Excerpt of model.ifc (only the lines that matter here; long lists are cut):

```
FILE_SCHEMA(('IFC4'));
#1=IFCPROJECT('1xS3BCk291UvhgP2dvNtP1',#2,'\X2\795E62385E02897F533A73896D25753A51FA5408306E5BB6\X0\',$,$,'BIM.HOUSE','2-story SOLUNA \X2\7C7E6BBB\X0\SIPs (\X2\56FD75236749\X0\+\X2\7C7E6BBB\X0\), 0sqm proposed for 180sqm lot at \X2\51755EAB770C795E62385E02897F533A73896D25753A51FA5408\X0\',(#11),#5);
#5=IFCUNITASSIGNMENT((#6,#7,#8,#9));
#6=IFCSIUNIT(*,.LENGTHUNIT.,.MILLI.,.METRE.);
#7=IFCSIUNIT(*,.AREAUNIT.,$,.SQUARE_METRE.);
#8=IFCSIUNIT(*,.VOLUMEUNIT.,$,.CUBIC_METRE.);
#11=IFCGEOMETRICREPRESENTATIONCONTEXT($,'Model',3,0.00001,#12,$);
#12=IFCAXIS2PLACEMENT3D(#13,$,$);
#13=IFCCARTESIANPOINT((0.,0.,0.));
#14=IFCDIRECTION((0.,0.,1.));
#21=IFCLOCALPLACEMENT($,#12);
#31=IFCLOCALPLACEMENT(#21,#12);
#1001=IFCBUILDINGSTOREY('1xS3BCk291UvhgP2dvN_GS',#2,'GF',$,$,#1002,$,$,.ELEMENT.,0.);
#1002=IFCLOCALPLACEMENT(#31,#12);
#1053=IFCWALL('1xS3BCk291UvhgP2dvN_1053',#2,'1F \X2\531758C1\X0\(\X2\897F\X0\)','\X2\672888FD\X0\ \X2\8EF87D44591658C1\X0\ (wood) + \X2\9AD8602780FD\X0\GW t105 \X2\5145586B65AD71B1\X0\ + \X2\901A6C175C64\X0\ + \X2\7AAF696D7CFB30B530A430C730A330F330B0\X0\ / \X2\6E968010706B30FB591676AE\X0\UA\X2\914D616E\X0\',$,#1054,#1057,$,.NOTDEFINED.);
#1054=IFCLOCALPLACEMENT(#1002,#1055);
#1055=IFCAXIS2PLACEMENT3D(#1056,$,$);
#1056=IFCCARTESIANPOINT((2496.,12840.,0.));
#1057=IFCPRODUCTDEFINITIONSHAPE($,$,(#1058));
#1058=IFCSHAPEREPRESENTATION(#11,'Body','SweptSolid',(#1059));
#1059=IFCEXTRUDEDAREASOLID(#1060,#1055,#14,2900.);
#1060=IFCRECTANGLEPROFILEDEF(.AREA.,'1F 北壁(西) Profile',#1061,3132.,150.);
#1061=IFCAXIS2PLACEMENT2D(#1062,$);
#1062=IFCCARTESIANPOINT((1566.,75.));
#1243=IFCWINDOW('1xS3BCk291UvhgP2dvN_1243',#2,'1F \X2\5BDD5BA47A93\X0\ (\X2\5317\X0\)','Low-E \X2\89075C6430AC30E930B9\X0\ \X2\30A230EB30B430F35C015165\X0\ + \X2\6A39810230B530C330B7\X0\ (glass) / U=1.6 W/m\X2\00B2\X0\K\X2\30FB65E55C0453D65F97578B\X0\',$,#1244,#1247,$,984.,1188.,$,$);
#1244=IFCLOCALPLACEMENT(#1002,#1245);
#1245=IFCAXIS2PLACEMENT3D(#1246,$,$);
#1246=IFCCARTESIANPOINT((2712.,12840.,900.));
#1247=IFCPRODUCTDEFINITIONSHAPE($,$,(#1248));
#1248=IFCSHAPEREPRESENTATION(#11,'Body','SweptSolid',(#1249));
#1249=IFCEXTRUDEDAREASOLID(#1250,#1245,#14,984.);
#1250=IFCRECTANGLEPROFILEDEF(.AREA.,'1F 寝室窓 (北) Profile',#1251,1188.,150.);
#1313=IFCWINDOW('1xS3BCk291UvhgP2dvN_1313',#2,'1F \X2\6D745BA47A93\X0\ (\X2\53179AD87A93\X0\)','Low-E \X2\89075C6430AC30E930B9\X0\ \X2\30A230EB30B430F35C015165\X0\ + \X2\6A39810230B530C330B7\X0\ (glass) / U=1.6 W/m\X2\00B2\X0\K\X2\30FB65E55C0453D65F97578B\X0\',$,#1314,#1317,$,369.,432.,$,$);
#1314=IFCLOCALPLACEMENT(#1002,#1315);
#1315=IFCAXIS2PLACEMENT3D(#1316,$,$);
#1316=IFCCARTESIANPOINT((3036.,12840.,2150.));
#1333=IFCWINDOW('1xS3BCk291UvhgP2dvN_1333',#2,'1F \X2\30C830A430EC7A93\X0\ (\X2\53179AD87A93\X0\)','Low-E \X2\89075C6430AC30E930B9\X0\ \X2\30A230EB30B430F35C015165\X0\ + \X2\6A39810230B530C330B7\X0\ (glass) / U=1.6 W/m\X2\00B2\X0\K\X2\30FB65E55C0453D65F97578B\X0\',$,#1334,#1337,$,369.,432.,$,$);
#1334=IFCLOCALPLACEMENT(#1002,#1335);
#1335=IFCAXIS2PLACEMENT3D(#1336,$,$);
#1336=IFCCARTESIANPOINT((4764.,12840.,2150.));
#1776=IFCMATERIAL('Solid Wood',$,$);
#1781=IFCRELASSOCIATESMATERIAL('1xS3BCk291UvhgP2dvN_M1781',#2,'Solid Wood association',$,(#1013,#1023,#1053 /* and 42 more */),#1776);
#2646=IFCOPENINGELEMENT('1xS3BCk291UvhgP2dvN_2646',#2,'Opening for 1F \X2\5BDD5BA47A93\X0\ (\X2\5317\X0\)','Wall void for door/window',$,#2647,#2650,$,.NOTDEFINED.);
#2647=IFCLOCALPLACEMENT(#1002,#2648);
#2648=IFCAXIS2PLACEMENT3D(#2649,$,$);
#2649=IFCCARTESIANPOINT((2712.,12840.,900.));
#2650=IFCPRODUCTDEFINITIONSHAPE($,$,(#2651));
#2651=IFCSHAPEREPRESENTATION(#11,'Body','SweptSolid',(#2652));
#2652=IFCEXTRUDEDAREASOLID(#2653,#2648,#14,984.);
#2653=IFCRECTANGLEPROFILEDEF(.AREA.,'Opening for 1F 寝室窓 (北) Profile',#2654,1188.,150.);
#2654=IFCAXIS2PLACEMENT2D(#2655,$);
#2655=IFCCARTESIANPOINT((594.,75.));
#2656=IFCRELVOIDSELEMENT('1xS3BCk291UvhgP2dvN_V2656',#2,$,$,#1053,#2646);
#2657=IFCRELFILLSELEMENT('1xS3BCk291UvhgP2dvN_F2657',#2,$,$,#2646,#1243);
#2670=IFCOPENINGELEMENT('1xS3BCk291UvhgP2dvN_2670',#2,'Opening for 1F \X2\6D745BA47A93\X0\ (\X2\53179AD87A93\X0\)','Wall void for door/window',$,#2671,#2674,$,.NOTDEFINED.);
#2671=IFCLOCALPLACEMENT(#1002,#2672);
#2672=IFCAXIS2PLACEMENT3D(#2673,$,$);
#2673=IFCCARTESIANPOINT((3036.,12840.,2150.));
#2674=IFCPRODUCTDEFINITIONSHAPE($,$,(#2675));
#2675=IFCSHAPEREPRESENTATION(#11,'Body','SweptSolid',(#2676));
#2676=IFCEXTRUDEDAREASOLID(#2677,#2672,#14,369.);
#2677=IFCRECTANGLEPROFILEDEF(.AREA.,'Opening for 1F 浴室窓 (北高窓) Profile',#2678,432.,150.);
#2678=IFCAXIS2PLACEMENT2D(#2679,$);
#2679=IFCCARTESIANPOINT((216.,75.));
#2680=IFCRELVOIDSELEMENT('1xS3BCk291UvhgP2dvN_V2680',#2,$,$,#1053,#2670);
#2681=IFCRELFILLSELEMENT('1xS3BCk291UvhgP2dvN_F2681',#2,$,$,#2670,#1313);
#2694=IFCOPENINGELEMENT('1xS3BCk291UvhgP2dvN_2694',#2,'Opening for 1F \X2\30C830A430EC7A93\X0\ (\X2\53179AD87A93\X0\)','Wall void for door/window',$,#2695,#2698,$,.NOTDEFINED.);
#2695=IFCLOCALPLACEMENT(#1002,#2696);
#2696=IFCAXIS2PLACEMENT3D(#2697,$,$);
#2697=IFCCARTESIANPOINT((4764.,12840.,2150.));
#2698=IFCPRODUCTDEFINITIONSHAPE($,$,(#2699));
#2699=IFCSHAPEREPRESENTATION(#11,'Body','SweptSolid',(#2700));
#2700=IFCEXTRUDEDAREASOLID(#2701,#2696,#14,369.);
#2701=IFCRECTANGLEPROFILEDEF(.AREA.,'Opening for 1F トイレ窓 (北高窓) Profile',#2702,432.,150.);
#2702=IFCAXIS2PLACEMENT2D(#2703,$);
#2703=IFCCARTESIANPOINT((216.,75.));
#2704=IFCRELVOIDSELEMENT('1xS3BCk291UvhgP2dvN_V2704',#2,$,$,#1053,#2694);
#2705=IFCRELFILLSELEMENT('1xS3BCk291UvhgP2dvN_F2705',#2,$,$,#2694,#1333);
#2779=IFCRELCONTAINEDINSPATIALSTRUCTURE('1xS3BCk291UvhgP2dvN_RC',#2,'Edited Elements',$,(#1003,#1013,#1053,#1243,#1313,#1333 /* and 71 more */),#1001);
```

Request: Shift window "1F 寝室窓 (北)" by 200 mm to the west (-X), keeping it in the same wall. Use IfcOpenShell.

```python
import ifcopenshell
import ifcopenshell.api.geometry
import ifcopenshell.util.placement

model = ifcopenshell.open("model.ifc")

window = model.by_id(1243)
opening = window.FillsVoids[0].RelatingOpeningElement
wall = opening.VoidsElements[0].RelatingBuildingElement

wall_matrix = ifcopenshell.util.placement.get_local_placement(wall.ObjectPlacement)
shift = wall_matrix[:3, 0] * -200.0
before = ifcopenshell.util.placement.get_local_placement(window.ObjectPlacement)[:3, 3].copy()

# The window is not placed relative to its opening, so move both.
for product in (opening, window):
    matrix = ifcopenshell.util.placement.get_local_placement(product.ObjectPlacement)
    matrix[:3, 3] += shift
    ifcopenshell.api.geometry.edit_object_placement(model, product=product, matrix=matrix, is_si=False)

after = ifcopenshell.util.placement.get_local_placement(window.ObjectPlacement)[:3, 3]
print("window moved by", (after - before).round(3) + 0.0)

model.write("model_updated.ifc")
```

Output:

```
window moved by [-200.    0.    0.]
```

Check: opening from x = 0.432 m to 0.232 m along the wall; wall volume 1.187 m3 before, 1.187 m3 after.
